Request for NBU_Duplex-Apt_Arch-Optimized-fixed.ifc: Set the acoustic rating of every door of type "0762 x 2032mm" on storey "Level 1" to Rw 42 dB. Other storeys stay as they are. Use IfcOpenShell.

First a look at what the model holds.

```python
import ifcopenshell
import ifcopenshell.util.element

model = ifcopenshell.open("NBU_Duplex-Apt_Arch-Optimized-fixed.ifc")
print(model.schema)
storey = next(s for s in model.by_type("IfcBuildingStorey") if s.Name == "Level 1")
doors = [e for e in ifcopenshell.util.element.get_decomposition(storey) if e.is_a("IfcDoor")]
seen = {}
for e in doors:
    element_type = ifcopenshell.util.element.get_type(e)
    key = (element_type.Name if element_type != e and element_type else None, ifcopenshell.util.element.get_pset(e, "Pset_DoorCommon", "AcousticRating"))
    seen[key] = seen.get(key, 0) + 1
for (name, value), count in sorted(seen.items(), key=str):
    print(count, "x", name, "|", value)
```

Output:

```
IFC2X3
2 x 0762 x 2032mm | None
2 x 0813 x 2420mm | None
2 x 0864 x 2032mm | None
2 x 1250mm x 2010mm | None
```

```python
import ifcopenshell
import ifcopenshell.api.pset
import ifcopenshell.util.element

model = ifcopenshell.open("NBU_Duplex-Apt_Arch-Optimized-fixed.ifc")

storey = next(s for s in model.by_type("IfcBuildingStorey") if s.Name == "Level 1")
doors = [e for e in ifcopenshell.util.element.get_decomposition(storey) if e.is_a("IfcDoor")]

count = 0
for e in doors:
    element_type = ifcopenshell.util.element.get_type(e)
    if element_type in (None, e) or element_type.Name != "0762 x 2032mm":
        continue
    # add_pset returns the element's existing set when there is one.
    pset = ifcopenshell.api.pset.add_pset(model, product=e, name="Pset_DoorCommon")
    ifcopenshell.api.pset.edit_pset(model, pset=pset, properties={"AcousticRating": "Rw 42 dB"})
    count += 1

print(count, "doors updated")

model.write("NBU_Duplex-Apt_Arch-Optimized-fixed_updated.ifc")
```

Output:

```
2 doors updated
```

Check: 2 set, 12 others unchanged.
